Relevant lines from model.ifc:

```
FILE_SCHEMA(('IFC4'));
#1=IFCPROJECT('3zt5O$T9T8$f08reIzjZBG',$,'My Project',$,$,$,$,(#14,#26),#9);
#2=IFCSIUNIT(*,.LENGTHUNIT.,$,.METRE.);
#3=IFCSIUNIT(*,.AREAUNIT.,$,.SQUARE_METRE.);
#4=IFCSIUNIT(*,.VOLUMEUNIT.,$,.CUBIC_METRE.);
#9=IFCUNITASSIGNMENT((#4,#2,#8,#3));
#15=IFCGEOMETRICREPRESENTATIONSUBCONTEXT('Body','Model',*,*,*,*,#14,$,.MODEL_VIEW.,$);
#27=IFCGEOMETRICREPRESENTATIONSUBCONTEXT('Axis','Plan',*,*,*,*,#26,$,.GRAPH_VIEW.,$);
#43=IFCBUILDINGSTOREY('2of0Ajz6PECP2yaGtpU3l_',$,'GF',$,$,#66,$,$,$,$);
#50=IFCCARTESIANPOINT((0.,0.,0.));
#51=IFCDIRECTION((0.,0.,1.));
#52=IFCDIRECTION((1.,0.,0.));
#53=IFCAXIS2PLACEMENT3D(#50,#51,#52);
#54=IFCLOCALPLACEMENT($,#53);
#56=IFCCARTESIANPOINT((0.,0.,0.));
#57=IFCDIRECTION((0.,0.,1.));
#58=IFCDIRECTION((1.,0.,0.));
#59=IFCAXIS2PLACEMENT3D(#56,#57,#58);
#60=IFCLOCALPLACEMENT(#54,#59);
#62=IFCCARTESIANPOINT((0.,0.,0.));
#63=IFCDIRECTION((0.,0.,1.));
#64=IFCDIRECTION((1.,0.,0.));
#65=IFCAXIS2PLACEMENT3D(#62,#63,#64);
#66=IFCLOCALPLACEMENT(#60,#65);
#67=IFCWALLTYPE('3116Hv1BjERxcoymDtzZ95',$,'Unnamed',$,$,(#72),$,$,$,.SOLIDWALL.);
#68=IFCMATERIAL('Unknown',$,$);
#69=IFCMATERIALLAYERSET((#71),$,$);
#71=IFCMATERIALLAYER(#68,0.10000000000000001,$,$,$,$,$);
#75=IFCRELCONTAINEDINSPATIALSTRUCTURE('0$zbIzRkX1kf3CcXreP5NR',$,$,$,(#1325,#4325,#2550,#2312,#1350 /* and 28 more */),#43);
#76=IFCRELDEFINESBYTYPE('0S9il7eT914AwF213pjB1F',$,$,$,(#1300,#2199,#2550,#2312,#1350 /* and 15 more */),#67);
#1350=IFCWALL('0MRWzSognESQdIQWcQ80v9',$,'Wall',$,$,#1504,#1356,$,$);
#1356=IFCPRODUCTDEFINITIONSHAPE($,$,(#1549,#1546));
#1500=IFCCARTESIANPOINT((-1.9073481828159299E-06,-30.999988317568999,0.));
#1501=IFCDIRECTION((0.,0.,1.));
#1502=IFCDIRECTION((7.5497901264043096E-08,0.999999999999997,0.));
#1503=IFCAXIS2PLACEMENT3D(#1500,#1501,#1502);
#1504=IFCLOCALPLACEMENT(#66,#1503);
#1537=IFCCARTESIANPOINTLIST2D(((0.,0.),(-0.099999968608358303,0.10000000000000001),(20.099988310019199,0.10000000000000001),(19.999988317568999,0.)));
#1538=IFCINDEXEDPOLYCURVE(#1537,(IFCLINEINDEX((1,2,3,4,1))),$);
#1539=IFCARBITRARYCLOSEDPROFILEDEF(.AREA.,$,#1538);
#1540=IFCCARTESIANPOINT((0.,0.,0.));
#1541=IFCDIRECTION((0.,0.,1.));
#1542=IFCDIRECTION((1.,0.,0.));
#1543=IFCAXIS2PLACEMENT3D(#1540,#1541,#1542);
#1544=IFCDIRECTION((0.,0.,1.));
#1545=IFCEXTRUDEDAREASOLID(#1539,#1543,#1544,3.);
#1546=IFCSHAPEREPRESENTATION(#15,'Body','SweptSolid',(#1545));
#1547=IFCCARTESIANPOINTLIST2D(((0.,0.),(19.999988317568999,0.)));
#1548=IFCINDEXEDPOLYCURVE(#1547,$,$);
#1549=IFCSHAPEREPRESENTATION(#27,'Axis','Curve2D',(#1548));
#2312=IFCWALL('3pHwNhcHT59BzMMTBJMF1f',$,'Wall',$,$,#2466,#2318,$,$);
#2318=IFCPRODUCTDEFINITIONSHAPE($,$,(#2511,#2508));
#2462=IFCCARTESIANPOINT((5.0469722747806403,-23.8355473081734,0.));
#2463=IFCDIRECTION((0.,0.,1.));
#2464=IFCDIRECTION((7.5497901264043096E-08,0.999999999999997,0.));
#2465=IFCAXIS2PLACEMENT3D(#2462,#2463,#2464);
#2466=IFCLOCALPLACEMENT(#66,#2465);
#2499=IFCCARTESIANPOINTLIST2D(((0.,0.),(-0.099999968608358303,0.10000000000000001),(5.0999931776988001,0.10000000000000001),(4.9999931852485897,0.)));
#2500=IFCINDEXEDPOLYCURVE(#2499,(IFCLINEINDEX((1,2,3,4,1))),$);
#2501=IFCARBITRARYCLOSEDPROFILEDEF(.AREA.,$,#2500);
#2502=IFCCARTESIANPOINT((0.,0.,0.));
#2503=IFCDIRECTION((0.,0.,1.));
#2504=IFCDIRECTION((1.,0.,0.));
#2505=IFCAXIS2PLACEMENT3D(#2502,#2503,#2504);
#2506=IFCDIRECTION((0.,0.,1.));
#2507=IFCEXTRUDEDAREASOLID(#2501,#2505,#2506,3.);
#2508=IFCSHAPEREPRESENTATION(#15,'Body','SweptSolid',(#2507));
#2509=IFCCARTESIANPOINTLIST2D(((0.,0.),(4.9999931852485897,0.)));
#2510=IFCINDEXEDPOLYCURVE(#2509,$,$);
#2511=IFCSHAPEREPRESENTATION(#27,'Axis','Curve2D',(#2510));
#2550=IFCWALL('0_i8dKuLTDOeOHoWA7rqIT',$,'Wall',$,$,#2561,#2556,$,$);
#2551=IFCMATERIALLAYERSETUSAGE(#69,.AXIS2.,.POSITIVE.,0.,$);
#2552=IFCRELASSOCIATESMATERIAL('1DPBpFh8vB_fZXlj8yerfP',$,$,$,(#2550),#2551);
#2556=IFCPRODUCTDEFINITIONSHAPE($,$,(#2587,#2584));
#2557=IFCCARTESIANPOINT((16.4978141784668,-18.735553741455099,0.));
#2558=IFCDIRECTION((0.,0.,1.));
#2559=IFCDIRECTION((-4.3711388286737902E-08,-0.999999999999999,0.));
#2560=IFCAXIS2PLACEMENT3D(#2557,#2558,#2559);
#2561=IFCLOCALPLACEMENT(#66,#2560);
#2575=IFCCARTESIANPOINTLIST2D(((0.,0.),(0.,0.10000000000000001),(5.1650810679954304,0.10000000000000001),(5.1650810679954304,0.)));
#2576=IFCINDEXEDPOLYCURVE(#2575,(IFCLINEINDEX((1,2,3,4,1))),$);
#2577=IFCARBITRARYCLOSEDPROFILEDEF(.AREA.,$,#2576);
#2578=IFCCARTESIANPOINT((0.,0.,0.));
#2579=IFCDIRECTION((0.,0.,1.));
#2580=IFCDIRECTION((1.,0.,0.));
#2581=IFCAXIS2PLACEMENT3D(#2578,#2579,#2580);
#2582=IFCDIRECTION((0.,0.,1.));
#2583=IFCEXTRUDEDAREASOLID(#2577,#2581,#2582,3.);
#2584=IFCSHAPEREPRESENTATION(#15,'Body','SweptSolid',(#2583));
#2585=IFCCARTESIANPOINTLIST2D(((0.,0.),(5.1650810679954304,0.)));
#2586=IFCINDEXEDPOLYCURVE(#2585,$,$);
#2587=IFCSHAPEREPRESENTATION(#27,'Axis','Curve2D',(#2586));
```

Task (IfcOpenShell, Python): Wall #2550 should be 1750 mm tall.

```python
import ifcopenshell
import ifcopenshell.geom
import ifcopenshell.util.representation
import ifcopenshell.util.shape
import ifcopenshell.util.unit

model = ifcopenshell.open("model.ifc")
unit_scale = ifcopenshell.util.unit.calculate_unit_scale(model)
settings = ifcopenshell.geom.settings()


def volume(element):
    """Net volume in cubic metres, openings subtracted."""
    shape = ifcopenshell.geom.create_shape(settings, element)
    return ifcopenshell.util.shape.get_volume(shape.geometry)


wall = model.by_guid("0_i8dKuLTDOeOHoWA7rqIT")
before = volume(wall)

body = ifcopenshell.util.representation.get_representation(wall, "Model", "Body")
solid = body.Items[0]
old_height = solid.Depth
solid.Depth = 1.75 / unit_scale
after = volume(wall)

print(f"height {old_height:g} -> {solid.Depth:g}, volume {before:.3f} -> {after:.3f} m3")

model.write("model_edited.ifc")
```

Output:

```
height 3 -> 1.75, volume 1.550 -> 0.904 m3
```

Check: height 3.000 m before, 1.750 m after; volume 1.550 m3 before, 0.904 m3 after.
